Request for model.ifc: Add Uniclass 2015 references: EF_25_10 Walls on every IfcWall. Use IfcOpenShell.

First a look at what the model holds.

```python
import ifcopenshell

model = ifcopenshell.open("model.ifc")
print(model.schema)
print("classifications:", [c.Name for c in model.by_type("IfcClassification")])
for ifc_class in ("IfcDoor", "IfcRoof", "IfcStair", "IfcWall", "IfcWindow"):
    print(ifc_class, len(model.by_type(ifc_class)))
```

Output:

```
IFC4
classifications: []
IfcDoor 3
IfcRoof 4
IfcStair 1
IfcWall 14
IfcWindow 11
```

```python
import ifcopenshell
import ifcopenshell.api.classification

model = ifcopenshell.open("model.ifc")

system = ifcopenshell.api.classification.add_classification(model, classification="Uniclass 2015")

codes = {
    "IfcWall": ("EF_25_10", "Walls"),
}
for ifc_class, (code, name) in codes.items():
    products = model.by_type(ifc_class)
    ifcopenshell.api.classification.add_reference(
        model, products=products, classification=system, identification=code, name=name
    )
    print(code, len(products))

model.write("model_edited.ifc")
```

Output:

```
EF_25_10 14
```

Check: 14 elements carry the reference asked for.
